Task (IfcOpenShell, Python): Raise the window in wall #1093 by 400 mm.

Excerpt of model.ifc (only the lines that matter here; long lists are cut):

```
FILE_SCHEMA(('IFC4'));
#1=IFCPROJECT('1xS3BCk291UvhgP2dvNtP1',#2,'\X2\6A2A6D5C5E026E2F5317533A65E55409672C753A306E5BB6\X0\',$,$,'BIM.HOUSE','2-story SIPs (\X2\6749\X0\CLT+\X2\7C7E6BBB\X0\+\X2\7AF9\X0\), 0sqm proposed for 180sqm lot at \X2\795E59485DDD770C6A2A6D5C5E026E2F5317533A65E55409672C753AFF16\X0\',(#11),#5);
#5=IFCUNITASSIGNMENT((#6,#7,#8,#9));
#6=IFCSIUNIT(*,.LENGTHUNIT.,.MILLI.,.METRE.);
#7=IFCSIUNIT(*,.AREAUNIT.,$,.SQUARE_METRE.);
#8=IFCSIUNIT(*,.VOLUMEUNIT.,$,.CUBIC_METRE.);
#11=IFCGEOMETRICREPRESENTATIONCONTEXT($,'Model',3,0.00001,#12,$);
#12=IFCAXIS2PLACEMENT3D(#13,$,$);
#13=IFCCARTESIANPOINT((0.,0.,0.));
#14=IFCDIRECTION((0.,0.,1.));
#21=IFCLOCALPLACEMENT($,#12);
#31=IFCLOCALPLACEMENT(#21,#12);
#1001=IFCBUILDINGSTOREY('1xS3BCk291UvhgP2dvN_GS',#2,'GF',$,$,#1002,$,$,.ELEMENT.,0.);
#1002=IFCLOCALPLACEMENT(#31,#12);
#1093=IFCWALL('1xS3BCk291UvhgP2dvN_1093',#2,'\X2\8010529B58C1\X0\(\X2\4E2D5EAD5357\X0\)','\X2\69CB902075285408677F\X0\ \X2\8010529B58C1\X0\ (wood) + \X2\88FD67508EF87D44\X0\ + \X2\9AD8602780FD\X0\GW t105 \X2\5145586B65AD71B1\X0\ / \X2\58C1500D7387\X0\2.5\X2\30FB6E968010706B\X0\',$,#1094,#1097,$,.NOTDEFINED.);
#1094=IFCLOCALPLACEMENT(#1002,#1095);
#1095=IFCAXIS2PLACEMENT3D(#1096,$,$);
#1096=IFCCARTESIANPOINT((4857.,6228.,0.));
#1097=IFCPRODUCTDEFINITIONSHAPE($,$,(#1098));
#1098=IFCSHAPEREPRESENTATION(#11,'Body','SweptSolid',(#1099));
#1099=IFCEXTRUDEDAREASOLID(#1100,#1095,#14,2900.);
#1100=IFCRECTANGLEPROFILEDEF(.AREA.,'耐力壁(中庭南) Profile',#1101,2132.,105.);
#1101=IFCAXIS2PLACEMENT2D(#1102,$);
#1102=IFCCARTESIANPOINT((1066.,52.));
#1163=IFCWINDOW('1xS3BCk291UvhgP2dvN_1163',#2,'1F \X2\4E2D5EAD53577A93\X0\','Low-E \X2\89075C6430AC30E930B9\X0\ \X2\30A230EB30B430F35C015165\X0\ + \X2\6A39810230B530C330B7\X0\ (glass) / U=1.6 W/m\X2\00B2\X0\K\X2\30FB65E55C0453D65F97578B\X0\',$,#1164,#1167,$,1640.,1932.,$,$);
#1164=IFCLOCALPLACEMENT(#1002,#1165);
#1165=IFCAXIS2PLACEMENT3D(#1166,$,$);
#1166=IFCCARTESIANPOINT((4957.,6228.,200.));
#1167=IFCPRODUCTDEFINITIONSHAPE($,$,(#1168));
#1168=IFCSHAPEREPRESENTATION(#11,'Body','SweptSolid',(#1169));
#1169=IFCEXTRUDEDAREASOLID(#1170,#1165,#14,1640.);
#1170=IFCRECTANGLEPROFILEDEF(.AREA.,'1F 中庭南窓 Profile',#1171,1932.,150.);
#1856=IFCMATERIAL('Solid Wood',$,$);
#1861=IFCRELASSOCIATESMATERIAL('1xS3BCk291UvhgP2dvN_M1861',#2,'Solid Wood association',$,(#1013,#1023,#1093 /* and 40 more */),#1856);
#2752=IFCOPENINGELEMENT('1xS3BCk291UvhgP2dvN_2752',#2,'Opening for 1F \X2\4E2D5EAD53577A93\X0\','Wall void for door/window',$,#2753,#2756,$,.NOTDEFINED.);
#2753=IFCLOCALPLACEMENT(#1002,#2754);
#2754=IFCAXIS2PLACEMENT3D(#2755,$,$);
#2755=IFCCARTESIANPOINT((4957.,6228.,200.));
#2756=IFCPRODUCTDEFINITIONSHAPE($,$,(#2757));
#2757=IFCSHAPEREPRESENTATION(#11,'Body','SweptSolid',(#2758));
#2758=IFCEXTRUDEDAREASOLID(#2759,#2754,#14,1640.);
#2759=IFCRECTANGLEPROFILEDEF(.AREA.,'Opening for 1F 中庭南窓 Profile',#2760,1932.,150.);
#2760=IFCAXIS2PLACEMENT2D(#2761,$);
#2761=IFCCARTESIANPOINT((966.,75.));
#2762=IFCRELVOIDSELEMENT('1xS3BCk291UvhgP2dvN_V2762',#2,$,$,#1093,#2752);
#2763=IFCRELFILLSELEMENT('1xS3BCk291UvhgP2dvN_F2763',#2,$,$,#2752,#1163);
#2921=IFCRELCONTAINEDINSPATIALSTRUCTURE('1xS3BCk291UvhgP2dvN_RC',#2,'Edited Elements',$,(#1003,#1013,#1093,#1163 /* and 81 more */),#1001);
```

```python
import numpy as np
import ifcopenshell
import ifcopenshell.api.geometry
import ifcopenshell.util.placement
import ifcopenshell.util.unit

model = ifcopenshell.open("model.ifc")
unit_scale = ifcopenshell.util.unit.calculate_unit_scale(model)

window = model.by_guid("1xS3BCk291UvhgP2dvN_1163")
opening = window.FillsVoids[0].RelatingOpeningElement
dz = 0.4 / unit_scale

shift = np.array([0.0, 0.0, dz])
# The window is not placed relative to its opening, so move both.
for product in (opening, window):
    matrix = ifcopenshell.util.placement.get_local_placement(product.ObjectPlacement)
    matrix[:3, 3] += shift
    ifcopenshell.api.geometry.edit_object_placement(model, product=product, matrix=matrix, is_si=False)

print(f"moved by {dz * unit_scale:+.3f} m")

model.write("model_edited.ifc")
```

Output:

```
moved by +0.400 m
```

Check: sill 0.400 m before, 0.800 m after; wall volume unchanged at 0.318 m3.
